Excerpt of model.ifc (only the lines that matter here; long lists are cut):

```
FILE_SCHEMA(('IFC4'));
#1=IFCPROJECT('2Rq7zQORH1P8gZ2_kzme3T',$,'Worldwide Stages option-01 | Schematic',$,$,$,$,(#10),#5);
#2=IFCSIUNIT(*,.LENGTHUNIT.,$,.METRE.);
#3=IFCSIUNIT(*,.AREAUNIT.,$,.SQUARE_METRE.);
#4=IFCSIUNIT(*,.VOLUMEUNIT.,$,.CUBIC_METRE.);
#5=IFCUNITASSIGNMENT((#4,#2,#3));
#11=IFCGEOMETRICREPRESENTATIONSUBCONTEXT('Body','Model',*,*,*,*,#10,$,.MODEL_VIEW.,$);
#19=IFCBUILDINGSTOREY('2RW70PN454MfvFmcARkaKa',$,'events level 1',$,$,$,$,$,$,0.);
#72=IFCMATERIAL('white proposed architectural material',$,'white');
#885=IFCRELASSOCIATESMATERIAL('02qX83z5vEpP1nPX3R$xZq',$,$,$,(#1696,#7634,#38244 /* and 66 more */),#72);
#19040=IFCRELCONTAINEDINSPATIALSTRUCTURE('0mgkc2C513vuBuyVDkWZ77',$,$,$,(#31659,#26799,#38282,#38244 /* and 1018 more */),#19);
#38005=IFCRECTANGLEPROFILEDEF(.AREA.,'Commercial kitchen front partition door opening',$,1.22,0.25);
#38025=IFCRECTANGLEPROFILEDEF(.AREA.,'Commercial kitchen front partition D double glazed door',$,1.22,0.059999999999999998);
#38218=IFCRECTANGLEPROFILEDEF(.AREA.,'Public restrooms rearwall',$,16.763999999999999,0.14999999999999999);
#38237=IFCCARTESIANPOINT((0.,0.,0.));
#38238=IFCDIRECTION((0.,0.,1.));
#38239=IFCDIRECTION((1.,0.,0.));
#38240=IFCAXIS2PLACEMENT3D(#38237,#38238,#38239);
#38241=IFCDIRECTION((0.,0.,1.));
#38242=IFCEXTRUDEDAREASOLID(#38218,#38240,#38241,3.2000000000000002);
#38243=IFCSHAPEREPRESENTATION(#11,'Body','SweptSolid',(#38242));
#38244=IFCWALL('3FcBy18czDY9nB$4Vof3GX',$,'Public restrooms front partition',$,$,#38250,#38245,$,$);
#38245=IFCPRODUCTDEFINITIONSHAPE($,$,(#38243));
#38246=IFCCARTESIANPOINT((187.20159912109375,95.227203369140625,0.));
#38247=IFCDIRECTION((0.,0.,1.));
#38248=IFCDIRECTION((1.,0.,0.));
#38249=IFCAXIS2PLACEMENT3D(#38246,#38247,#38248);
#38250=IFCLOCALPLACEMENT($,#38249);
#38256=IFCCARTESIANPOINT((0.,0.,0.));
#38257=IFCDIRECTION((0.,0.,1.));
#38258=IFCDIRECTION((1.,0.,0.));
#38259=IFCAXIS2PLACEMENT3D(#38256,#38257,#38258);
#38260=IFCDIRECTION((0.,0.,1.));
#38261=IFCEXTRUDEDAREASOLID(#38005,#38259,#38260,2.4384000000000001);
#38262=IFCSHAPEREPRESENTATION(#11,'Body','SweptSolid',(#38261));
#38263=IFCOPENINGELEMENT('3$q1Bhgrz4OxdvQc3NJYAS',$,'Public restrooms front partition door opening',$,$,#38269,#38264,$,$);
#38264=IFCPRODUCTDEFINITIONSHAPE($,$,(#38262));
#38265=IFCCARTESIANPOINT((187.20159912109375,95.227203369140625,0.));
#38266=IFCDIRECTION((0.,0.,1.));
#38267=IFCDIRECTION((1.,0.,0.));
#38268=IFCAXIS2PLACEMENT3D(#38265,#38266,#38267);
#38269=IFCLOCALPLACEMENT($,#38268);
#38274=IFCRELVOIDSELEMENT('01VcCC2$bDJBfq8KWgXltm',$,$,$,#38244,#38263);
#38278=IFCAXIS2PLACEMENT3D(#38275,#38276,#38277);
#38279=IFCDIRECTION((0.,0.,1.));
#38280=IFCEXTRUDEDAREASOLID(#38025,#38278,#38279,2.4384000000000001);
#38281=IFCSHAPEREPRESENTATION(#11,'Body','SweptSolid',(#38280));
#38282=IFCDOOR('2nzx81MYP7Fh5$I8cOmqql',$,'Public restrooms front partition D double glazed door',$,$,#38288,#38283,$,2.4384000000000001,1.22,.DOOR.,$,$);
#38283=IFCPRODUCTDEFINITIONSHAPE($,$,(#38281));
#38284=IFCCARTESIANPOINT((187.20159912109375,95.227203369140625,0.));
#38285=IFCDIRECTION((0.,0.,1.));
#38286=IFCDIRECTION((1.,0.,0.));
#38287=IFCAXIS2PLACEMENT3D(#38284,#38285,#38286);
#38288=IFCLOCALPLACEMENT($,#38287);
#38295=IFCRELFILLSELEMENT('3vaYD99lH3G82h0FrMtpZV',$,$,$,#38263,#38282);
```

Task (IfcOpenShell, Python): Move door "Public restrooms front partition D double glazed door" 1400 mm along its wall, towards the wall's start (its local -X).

```python
import ifcopenshell
import ifcopenshell.api.geometry
import ifcopenshell.util.placement

model = ifcopenshell.open("model.ifc")

door = model.by_guid("2nzx81MYP7Fh5$I8cOmqql")
opening = door.FillsVoids[0].RelatingOpeningElement
wall = opening.VoidsElements[0].RelatingBuildingElement

wall_matrix = ifcopenshell.util.placement.get_local_placement(wall.ObjectPlacement)
shift = wall_matrix[:3, 0] * -1.4
before = ifcopenshell.util.placement.get_local_placement(door.ObjectPlacement)[:3, 3].copy()

# The door is not placed relative to its opening, so move both.
for product in (opening, door):
    matrix = ifcopenshell.util.placement.get_local_placement(product.ObjectPlacement)
    matrix[:3, 3] += shift
    ifcopenshell.api.geometry.edit_object_placement(model, product=product, matrix=matrix, is_si=False)

after = ifcopenshell.util.placement.get_local_placement(door.ObjectPlacement)[:3, 3]
print("door moved by", (after - before).round(3) + 0.0)

model.write("model_v2.ifc")
```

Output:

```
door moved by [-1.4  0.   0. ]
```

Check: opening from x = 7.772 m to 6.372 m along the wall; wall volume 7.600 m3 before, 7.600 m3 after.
